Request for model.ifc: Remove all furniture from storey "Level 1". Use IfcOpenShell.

First a look at what the model holds.

```python
import ifcopenshell
import ifcopenshell.util.element

model = ifcopenshell.open("model.ifc")
print(model.schema)
storey = next(s for s in model.by_type("IfcBuildingStorey") if s.Name == "Level 1")
furniture = [e for e in ifcopenshell.util.element.get_decomposition(storey) if e.is_a("IfcFurnishingElement")]
seen = {}
for e in furniture:
    element_type = ifcopenshell.util.element.get_type(e)
    name = element_type.Name if element_type not in (None, e) else None
    seen[name] = seen.get(name, 0) + 1
for name, count in sorted(seen.items(), key=str):
    print(count, "x", name)
```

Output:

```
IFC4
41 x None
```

```python
import ifcopenshell
import ifcopenshell.api.root
import ifcopenshell.util.element

model = ifcopenshell.open("model.ifc")

storey = next(s for s in model.by_type("IfcBuildingStorey") if s.Name == "Level 1")
furniture = [e for e in ifcopenshell.util.element.get_decomposition(storey) if e.is_a("IfcFurnishingElement")]

for e in furniture:
    ifcopenshell.api.root.remove_product(model, product=e)
print(len(furniture), "removed")

model.write("model_updated.ifc")
```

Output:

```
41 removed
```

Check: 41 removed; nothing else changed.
